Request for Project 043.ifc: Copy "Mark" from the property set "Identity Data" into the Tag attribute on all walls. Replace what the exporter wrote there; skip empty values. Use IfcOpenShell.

First a look at what the model holds.

```python
import ifcopenshell
import ifcopenshell.util.element

model = ifcopenshell.open("Project 043.ifc")
print(model.schema)
walls = model.by_type("IfcWall")
print(len(walls), "walls")
for e in walls[:8]:
    source = ifcopenshell.util.element.get_pset(e, "Identity Data", "Mark")
    target = e.Tag
    print(e.id(), repr(source), repr(target), sep=" | ")
```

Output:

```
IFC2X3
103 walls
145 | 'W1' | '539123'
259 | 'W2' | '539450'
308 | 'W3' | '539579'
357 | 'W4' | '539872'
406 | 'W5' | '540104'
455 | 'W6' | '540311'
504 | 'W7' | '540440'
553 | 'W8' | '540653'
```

```python
import ifcopenshell
import ifcopenshell.util.element

model = ifcopenshell.open("Project 043.ifc")

count = 0
for e in model.by_type("IfcWall"):
    value = ifcopenshell.util.element.get_pset(e, "Identity Data", "Mark")
    current = e.Tag
    if not value or not value.strip() or current == value:
        continue
    e.Tag = value
    count += 1

print(count, "walls updated")

model.write("Project 043_edited.ifc")
```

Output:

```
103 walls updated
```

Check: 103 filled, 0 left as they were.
